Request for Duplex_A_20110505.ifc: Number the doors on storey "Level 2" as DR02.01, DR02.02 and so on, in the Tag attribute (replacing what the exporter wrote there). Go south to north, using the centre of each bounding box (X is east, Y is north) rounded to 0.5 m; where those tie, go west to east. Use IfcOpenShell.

First a look at what the model holds.

```python
import ifcopenshell
import ifcopenshell.util.element
import ifcopenshell.util.placement

model = ifcopenshell.open("Duplex_A_20110505.ifc")
print(model.schema)
storey = next(s for s in model.by_type("IfcBuildingStorey") if s.Name == "Level 2")
doors = [e for e in ifcopenshell.util.element.get_decomposition(storey) if e.is_a("IfcDoor")]
for e in sorted(doors, key=lambda e: e.id()):
    origin = ifcopenshell.util.placement.get_local_placement(e.ObjectPlacement)[:3, 3]
    print(e.id(), e.Tag, e.Name, origin.round(2) + 0.0, sep=" | ")
```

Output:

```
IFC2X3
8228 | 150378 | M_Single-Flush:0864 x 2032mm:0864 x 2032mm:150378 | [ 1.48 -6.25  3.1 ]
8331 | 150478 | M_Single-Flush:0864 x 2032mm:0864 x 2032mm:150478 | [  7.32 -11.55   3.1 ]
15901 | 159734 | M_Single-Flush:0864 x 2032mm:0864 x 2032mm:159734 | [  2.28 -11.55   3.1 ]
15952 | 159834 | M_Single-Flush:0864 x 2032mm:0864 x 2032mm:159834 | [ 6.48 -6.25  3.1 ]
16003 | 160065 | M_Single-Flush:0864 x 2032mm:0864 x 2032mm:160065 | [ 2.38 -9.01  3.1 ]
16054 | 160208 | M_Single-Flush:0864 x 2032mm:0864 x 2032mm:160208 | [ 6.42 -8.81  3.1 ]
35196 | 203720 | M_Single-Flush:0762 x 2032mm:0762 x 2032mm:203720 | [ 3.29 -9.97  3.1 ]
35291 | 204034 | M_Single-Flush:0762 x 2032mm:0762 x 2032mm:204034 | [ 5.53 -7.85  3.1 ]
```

```python
import ifcopenshell
import ifcopenshell.geom
import ifcopenshell.util.element
import ifcopenshell.util.shape

model = ifcopenshell.open("Duplex_A_20110505.ifc")
settings = ifcopenshell.geom.settings()
settings.set("use-world-coords", True)


def centre(element):
    shape = ifcopenshell.geom.create_shape(settings, element)
    return ifcopenshell.util.shape.get_bbox_centroid(shape.geometry)


storey = next(s for s in model.by_type("IfcBuildingStorey") if s.Name == "Level 2")
doors = [e for e in ifcopenshell.util.element.get_decomposition(storey) if e.is_a("IfcDoor")]

# Insertion points can sit at a corner or the storey origin, so sort by the geometry (in metres).
centres = {e: centre(e) for e in doors}
doors.sort(key=lambda e: (round(centres[e][1] / 0.5), centres[e][0]))

for i, e in enumerate(doors, start=1):
    number = f"DR02.{i:02d}"
    e.Tag = number
    print(e.id(), number)

model.write("Duplex_A_20110505_v2.ifc")
```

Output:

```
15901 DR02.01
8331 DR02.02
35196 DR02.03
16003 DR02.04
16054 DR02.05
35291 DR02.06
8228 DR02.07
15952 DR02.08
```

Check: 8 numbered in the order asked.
